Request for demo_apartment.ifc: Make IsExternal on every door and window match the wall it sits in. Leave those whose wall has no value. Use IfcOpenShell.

First a look at what the model holds.

```python
import ifcopenshell
import ifcopenshell.util.element

model = ifcopenshell.open("demo_apartment.ifc")
print(model.schema)
seen = {}
for e in model.by_type("IfcDoor") + model.by_type("IfcWindow"):
    if not e.FillsVoids:
        continue
    host = e.FillsVoids[0].RelatingOpeningElement.VoidsElements[0].RelatingBuildingElement
    own = ifcopenshell.util.element.get_pset(e, f"Pset_{e.is_a()[3:].removesuffix('StandardCase')}Common", "IsExternal")
    wall = ifcopenshell.util.element.get_pset(host, "Pset_WallCommon", "IsExternal")
    seen[e.is_a(), own, wall] = seen.get((e.is_a(), own, wall), 0) + 1
for (cls, own, wall), count in sorted(seen.items(), key=str):
    print(count, cls, "IsExternal:", own, "| host wall:", wall)
```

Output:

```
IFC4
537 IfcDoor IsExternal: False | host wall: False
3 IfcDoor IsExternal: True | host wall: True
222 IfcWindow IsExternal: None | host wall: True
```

```python
import ifcopenshell
import ifcopenshell.api.pset
import ifcopenshell.util.element

model = ifcopenshell.open("demo_apartment.ifc")

count = 0
for ifc_class, pset_name in (("IfcDoor", "Pset_DoorCommon"), ("IfcWindow", "Pset_WindowCommon")):
    for e in model.by_type(ifc_class):
        if not e.FillsVoids:
            continue
        host = e.FillsVoids[0].RelatingOpeningElement.VoidsElements[0].RelatingBuildingElement
        external = ifcopenshell.util.element.get_pset(host, "Pset_WallCommon", "IsExternal")
        if external is None or ifcopenshell.util.element.get_pset(e, pset_name, "IsExternal") == external:
            continue
        pset = ifcopenshell.api.pset.add_pset(model, product=e, name=pset_name)
        ifcopenshell.api.pset.edit_pset(model, pset=pset, properties={"IsExternal": external})
        count += 1

print(count, "updated")

model.write("demo_apartment_v2.ifc")
```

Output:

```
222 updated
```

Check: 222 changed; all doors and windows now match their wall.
